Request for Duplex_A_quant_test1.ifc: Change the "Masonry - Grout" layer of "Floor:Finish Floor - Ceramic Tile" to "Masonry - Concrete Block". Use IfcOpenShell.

First a look at what the model holds.

```python
import ifcopenshell
import ifcopenshell.util.element

model = ifcopenshell.open("Duplex_A_quant_test1.ifc")
print(model.schema)
for layer_set in model.by_type("IfcMaterialLayerSet"):
    if layer_set.LayerSetName == "Floor:Finish Floor - Ceramic Tile":
        for layer in layer_set.MaterialLayers:
            print(layer.id(), layer.Material and layer.Material.Name, layer.LayerThickness, sep=" | ")
        print(len(ifcopenshell.util.element.get_elements_by_material(model, layer_set)), "elements and types use it")
print(sorted(m.Name for m in model.by_type("IfcMaterial") if m.Name)[:60])
```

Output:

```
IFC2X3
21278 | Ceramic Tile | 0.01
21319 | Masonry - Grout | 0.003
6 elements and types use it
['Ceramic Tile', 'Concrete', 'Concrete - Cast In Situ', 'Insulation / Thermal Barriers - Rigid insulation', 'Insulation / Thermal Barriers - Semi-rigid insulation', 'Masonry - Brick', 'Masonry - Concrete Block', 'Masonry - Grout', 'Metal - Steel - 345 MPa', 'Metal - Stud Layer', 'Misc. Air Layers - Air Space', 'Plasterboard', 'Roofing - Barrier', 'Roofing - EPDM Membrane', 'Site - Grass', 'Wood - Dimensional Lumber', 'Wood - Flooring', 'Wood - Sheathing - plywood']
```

```python
import ifcopenshell
import ifcopenshell.api.material

model = ifcopenshell.open("Duplex_A_quant_test1.ifc")

layer_set = next(s for s in model.by_type("IfcMaterialLayerSet") if s.LayerSetName == "Floor:Finish Floor - Ceramic Tile")
layer = next(l for l in layer_set.MaterialLayers if l.Material and l.Material.Name == "Masonry - Grout")
material = next(m for m in model.by_type("IfcMaterial") if m.Name == "Masonry - Concrete Block")

# Point this one layer at the other material; renaming the old one would change it everywhere.
ifcopenshell.api.material.edit_layer(model, layer=layer, attributes={}, material=material)

print([l.Material.Name if l.Material else None for l in layer_set.MaterialLayers])

model.write("Duplex_A_quant_test1_rev.ifc")
```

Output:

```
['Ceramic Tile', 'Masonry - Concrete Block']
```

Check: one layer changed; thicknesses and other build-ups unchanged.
